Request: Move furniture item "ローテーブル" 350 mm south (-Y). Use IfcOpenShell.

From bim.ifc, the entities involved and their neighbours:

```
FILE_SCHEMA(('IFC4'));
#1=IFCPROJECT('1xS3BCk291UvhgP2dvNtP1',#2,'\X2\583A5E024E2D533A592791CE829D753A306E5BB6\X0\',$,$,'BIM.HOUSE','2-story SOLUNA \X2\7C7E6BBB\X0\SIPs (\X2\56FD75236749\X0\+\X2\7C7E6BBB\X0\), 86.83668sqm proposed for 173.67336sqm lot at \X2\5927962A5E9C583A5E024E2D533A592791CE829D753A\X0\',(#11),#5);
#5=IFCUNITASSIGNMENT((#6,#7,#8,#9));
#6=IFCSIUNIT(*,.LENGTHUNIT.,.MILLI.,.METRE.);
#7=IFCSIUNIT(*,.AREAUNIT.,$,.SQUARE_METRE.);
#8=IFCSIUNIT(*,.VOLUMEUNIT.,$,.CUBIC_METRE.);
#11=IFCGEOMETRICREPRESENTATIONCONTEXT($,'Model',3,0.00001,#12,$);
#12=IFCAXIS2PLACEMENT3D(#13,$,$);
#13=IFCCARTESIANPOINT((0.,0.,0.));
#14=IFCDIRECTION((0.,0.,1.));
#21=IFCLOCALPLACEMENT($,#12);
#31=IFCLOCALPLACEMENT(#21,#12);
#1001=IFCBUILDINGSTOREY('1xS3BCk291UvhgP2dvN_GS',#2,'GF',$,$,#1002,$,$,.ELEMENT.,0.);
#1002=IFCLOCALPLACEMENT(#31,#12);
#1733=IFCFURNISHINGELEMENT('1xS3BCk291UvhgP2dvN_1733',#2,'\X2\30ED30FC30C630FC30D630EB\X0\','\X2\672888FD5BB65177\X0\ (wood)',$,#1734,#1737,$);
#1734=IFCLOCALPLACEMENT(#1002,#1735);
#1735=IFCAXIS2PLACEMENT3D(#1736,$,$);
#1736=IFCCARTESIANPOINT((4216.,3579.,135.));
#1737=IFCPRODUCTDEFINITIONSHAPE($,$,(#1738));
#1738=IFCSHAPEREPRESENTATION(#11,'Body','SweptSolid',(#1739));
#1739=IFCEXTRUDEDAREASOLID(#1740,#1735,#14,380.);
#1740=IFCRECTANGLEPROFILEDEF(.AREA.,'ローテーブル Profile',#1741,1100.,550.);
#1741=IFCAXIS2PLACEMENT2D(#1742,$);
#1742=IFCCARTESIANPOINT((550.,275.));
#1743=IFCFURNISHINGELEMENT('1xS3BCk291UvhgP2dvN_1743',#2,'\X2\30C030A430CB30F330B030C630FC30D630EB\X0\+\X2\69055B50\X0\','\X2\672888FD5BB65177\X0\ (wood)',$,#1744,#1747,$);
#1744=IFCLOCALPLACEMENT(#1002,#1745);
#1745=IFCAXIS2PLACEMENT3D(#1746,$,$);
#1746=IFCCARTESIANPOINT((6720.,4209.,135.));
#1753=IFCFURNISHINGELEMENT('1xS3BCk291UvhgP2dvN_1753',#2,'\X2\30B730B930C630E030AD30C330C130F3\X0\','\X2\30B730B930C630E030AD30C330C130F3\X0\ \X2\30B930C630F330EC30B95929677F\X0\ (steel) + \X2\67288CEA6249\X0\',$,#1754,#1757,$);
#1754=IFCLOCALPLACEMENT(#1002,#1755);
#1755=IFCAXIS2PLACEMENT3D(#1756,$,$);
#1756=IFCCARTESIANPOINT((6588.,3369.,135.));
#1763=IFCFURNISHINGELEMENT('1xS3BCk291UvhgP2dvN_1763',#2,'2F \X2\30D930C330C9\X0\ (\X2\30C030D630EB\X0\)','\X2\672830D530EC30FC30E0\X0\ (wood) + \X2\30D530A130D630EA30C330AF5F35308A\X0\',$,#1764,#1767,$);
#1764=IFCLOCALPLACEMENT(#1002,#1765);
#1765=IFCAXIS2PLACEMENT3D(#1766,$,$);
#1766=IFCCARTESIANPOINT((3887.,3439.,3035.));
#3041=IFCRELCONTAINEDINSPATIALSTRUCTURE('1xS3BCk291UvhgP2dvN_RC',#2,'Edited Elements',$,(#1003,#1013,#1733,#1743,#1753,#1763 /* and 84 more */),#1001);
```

```python
import ifcopenshell
import ifcopenshell.api.geometry
import ifcopenshell.util.placement
import ifcopenshell.util.unit

model = ifcopenshell.open("bim.ifc")
unit_scale = ifcopenshell.util.unit.calculate_unit_scale(model)

item = model.by_id(1733)
matrix = ifcopenshell.util.placement.get_local_placement(item.ObjectPlacement)
matrix[1, 3] -= 0.35 / unit_scale
ifcopenshell.api.geometry.edit_object_placement(model, product=item, matrix=matrix, is_si=False)

print(ifcopenshell.util.placement.get_local_placement(item.ObjectPlacement).round(3) + 0.0)

model.write("bim_edited.ifc")
```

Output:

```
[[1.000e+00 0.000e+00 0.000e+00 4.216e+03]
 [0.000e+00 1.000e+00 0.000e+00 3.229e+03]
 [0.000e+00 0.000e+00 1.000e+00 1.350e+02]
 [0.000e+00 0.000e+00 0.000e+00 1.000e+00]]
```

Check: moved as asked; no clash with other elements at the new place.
